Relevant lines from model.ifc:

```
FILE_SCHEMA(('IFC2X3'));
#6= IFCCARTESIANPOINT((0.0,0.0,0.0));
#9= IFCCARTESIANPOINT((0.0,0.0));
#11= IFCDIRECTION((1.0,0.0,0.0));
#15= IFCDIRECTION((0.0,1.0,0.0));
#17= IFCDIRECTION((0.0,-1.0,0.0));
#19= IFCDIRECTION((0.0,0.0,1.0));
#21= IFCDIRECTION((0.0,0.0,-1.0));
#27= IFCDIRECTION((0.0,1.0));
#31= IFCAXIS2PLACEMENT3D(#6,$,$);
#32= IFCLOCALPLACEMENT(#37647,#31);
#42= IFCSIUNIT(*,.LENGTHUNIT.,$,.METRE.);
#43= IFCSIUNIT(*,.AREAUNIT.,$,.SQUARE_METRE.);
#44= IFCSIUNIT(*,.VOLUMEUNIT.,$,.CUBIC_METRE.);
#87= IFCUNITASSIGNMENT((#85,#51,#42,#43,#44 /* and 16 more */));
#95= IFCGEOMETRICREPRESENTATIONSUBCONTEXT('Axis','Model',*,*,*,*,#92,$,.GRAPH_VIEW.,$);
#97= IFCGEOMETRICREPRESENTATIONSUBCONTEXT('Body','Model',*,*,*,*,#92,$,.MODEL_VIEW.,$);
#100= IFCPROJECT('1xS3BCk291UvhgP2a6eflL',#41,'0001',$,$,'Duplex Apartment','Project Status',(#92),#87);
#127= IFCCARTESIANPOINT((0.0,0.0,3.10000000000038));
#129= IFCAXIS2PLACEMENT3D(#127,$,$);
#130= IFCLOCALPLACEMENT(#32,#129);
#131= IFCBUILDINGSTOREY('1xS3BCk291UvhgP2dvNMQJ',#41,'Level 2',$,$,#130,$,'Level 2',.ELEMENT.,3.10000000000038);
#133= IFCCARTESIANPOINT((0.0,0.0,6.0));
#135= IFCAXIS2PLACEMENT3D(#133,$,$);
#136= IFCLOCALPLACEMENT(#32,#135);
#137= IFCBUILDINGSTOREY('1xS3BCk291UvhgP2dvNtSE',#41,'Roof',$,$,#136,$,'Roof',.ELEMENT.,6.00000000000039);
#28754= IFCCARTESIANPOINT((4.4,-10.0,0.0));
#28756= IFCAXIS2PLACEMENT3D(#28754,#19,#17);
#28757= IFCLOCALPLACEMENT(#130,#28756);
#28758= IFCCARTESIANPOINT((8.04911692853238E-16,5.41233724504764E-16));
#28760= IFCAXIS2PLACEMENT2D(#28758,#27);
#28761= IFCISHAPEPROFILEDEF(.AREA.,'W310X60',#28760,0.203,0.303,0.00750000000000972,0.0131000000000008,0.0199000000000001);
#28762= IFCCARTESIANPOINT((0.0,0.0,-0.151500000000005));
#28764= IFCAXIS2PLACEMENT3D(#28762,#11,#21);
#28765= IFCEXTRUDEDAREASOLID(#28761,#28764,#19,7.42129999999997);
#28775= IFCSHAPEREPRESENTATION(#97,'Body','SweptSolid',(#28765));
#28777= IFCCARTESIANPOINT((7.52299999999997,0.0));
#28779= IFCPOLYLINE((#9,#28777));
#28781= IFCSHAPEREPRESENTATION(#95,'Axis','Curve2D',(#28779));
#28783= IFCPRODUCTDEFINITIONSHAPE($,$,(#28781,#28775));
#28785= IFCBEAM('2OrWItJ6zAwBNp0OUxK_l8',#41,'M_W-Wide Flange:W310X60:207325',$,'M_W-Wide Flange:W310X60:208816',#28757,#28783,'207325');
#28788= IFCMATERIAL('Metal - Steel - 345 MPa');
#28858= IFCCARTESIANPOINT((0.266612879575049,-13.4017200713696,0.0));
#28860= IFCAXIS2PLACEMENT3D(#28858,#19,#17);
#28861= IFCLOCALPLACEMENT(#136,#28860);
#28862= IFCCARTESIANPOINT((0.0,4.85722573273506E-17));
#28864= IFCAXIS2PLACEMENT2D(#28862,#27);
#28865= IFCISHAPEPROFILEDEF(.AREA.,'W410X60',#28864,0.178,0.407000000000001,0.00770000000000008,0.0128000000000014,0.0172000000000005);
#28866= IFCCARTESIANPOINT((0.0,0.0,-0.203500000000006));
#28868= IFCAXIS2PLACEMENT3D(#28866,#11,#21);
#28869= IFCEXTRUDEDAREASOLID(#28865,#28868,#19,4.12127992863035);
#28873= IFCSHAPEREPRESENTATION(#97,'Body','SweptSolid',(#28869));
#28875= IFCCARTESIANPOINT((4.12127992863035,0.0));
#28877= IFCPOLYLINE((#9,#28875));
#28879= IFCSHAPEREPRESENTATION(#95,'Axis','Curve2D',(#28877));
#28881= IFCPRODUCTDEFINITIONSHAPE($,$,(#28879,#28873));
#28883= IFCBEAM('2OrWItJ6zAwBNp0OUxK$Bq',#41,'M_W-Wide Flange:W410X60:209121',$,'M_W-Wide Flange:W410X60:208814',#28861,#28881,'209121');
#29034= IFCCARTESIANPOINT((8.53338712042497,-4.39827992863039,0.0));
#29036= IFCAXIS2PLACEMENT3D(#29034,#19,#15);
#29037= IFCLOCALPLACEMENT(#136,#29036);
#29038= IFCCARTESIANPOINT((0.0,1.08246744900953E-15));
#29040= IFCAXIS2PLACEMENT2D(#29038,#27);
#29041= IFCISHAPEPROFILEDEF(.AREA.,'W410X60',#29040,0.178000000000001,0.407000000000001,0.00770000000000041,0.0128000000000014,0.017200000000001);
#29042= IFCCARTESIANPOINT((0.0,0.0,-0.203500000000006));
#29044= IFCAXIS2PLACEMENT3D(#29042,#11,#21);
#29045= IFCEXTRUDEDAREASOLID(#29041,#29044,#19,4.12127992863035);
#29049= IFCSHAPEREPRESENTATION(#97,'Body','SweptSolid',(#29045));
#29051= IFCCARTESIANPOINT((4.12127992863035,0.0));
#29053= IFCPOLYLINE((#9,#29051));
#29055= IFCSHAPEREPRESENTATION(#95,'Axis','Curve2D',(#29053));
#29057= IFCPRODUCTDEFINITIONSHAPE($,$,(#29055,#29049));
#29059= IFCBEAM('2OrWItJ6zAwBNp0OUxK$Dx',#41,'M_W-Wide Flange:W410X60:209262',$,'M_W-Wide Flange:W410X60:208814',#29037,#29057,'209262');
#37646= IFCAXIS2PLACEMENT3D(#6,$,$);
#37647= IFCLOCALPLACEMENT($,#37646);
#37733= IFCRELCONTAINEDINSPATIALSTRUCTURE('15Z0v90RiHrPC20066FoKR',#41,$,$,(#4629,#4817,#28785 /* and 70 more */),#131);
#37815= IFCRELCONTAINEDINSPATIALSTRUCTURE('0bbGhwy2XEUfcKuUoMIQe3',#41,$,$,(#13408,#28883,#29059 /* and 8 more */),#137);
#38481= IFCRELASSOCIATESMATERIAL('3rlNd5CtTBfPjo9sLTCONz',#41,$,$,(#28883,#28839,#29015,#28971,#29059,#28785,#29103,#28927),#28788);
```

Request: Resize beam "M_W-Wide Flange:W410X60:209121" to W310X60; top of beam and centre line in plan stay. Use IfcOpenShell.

```python
import ifcopenshell
import ifcopenshell.util.element
import ifcopenshell.util.representation

model = ifcopenshell.open("model.ifc")

member = model.by_id(28883)
source = next(p for p in model.by_type("IfcIShapeProfileDef") if p.ProfileName == "W310X60")

body = ifcopenshell.util.representation.get_representation(member, "Model", "Body")
solid = body.Items[0]
old_profile = solid.SweptArea

# Copy the section's sizes but keep this member's own profile position.
profile = ifcopenshell.util.element.copy(model, source)
# Profiles are centred, so shift by half the change in depth to hold the top.
shift = (old_profile.OverallDepth - profile.OverallDepth) / 2
x, y = old_profile.Position.Location.Coordinates
up = (-1.0, 0.0)  # upwards, in the solid's own plane
location = model.createIfcCartesianPoint((x + up[0] * shift, y + up[1] * shift))
profile.Position = model.createIfcAxis2Placement2D(location, old_profile.Position.RefDirection)
solid.SweptArea = profile
if not model.get_total_inverses(old_profile):
    ifcopenshell.util.element.remove_deep2(model, old_profile)
member.Name = member.Name.replace("W410X60", "W310X60")
member.ObjectType = member.ObjectType.replace("W410X60", "W310X60")

print(solid.SweptArea)

model.write("model-out.ifc")
```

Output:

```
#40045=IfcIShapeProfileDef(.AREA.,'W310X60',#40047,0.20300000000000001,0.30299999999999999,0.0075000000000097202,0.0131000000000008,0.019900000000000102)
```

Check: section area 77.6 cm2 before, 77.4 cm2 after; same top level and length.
